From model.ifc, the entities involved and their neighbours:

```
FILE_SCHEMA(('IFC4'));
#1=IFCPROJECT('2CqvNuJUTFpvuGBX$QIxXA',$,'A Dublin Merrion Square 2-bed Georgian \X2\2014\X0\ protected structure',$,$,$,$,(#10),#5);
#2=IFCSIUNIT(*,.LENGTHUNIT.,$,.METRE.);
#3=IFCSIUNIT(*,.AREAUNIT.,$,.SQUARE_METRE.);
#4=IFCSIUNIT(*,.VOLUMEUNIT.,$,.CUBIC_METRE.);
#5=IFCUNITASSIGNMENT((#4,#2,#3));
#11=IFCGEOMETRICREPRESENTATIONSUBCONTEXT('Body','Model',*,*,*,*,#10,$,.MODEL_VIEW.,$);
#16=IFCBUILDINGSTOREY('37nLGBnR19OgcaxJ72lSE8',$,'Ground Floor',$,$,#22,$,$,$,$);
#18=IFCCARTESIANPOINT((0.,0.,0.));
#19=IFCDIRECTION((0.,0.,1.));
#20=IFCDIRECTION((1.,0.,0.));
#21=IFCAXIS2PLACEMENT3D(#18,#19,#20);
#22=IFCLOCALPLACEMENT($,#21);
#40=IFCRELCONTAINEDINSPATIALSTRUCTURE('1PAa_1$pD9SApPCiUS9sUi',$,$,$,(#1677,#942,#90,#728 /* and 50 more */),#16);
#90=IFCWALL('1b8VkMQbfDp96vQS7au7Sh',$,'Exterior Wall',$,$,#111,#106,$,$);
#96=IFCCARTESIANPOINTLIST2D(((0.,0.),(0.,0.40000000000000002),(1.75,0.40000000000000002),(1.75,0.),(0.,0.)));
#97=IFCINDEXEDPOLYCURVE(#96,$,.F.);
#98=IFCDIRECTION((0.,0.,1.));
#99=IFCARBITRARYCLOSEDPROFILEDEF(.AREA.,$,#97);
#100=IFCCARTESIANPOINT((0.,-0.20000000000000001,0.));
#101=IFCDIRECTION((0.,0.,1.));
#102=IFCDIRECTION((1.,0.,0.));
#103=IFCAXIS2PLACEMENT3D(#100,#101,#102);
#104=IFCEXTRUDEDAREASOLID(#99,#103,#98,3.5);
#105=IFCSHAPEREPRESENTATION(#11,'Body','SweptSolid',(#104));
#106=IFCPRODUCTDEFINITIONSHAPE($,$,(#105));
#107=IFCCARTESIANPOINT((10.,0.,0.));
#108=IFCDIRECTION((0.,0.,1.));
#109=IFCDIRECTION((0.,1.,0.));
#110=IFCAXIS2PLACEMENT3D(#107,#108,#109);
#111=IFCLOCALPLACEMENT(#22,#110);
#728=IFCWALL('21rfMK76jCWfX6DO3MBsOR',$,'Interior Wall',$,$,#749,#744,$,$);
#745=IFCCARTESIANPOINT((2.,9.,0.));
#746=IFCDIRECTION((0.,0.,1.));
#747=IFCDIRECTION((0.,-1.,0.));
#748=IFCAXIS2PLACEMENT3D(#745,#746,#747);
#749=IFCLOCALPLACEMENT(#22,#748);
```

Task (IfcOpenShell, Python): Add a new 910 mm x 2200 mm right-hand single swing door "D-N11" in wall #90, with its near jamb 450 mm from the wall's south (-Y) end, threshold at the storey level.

```python
import numpy as np
import ifcopenshell
import ifcopenshell.api.feature
import ifcopenshell.api.geometry
import ifcopenshell.api.root
import ifcopenshell.api.spatial
import ifcopenshell.geom
import ifcopenshell.util.element
import ifcopenshell.util.placement
import ifcopenshell.util.representation
import ifcopenshell.util.shape
import ifcopenshell.util.unit

model = ifcopenshell.open("model.ifc")
unit_scale = ifcopenshell.util.unit.calculate_unit_scale(model)
settings = ifcopenshell.geom.settings()


def volume(element):
    """Net volume in cubic metres, openings subtracted."""
    shape = ifcopenshell.geom.create_shape(settings, element)
    return ifcopenshell.util.shape.get_volume(shape.geometry)


wall = model.by_guid("1b8VkMQbfDp96vQS7au7Sh")
storey = ifcopenshell.util.element.get_container(wall, ifc_class="IfcBuildingStorey")
context = ifcopenshell.util.representation.get_context(model, "Model", "Body", "MODEL_VIEW")
before = volume(wall)

width, height, from_end, sill = 0.91, 2.2, 0.45, 0.0  # metres

# The wall runs along its own X axis, and the end named is its -X end.
wall_shape = ifcopenshell.geom.create_shape(settings, wall)
x, y, z = ifcopenshell.util.shape.get_vertices(wall_shape.geometry).T
start = x.min() + from_end
face, thickness = float(y.min()), float(y.max() - y.min())
wall_matrix = ifcopenshell.util.placement.get_local_placement(wall.ObjectPlacement)
level = ifcopenshell.util.placement.get_local_placement(storey.ObjectPlacement)[2, 3]


def in_wall(x, y):
    """Placement at x, y metres in the wall's axes, at sill height."""
    matrix = wall_matrix.copy()
    matrix[:, 3] = wall_matrix @ np.array([x / unit_scale, y / unit_scale, 0.0, 1.0])
    matrix[2, 3] = level + sill / unit_scale
    return matrix


# Opening: a box that overshoots both wall faces by 50 mm.
opening = ifcopenshell.api.root.create_entity(model, ifc_class="IfcOpeningElement", predefined_type="OPENING")
box = ifcopenshell.api.geometry.add_wall_representation(
    model, context=context, length=width, height=height, thickness=thickness + 0.1
)
ifcopenshell.api.geometry.assign_representation(model, product=opening, representation=box)
ifcopenshell.api.geometry.edit_object_placement(model, product=opening, matrix=in_wall(start, face - 0.05), is_si=False)
ifcopenshell.api.feature.add_feature(model, feature=opening, element=wall)

door = ifcopenshell.api.root.create_entity(model, ifc_class="IfcDoor", name="D-N11", predefined_type="DOOR")
door.OverallWidth, door.OverallHeight = width / unit_scale, height / unit_scale
door.OperationType = "SINGLE_SWING_RIGHT"
body = ifcopenshell.api.geometry.add_door_representation(
    model,
    context=context,
    overall_width=door.OverallWidth,
    overall_height=door.OverallHeight,
    operation_type="SINGLE_SWING_RIGHT",
    lining_properties={"LiningDepth": thickness / unit_scale, "ThresholdDepth": thickness / unit_scale},
)
ifcopenshell.api.geometry.assign_representation(model, product=door, representation=body)
ifcopenshell.api.spatial.assign_container(model, products=[door], relating_structure=storey)
ifcopenshell.api.feature.add_filling(model, opening=opening, element=door)

# The lining spans the wall, so the door starts at the wall face.
ifcopenshell.api.geometry.edit_object_placement(model, product=door, matrix=in_wall(start, face), is_si=False)

after = volume(wall)

print(f"wall volume {before:.3f} -> {after:.3f} m3")

model.write("model_v2.ifc")
```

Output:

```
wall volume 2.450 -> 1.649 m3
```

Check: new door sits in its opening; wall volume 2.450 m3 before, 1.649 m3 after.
